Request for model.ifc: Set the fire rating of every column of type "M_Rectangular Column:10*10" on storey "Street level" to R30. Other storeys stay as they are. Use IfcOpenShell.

First a look at what the model holds.

```python
import ifcopenshell
import ifcopenshell.util.element

model = ifcopenshell.open("model.ifc")
print(model.schema)
storey = next(s for s in model.by_type("IfcBuildingStorey") if s.Name == "Street level")
columns = [e for e in ifcopenshell.util.element.get_decomposition(storey) if e.is_a("IfcColumn")]
seen = {}
for e in columns:
    element_type = ifcopenshell.util.element.get_type(e)
    key = (element_type.Name if element_type != e and element_type else None, ifcopenshell.util.element.get_pset(e, "Pset_ColumnCommon", "FireRating"))
    seen[key] = seen.get(key, 0) + 1
for (name, value), count in sorted(seen.items(), key=str):
    print(count, "x", name, "|", value)
```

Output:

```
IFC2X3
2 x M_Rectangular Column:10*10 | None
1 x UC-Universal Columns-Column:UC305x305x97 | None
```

```python
import ifcopenshell
import ifcopenshell.api.pset
import ifcopenshell.util.element

model = ifcopenshell.open("model.ifc")

storey = next(s for s in model.by_type("IfcBuildingStorey") if s.Name == "Street level")
columns = [e for e in ifcopenshell.util.element.get_decomposition(storey) if e.is_a("IfcColumn")]

count = 0
for e in columns:
    element_type = ifcopenshell.util.element.get_type(e)
    if element_type in (None, e) or element_type.Name != "M_Rectangular Column:10*10":
        continue
    # add_pset returns the element's existing set when there is one.
    pset = ifcopenshell.api.pset.add_pset(model, product=e, name="Pset_ColumnCommon")
    ifcopenshell.api.pset.edit_pset(model, pset=pset, properties={"FireRating": "R30"})
    count += 1

print(count, "columns updated")

model.write("model_edited.ifc")
```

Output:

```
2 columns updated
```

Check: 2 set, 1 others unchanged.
